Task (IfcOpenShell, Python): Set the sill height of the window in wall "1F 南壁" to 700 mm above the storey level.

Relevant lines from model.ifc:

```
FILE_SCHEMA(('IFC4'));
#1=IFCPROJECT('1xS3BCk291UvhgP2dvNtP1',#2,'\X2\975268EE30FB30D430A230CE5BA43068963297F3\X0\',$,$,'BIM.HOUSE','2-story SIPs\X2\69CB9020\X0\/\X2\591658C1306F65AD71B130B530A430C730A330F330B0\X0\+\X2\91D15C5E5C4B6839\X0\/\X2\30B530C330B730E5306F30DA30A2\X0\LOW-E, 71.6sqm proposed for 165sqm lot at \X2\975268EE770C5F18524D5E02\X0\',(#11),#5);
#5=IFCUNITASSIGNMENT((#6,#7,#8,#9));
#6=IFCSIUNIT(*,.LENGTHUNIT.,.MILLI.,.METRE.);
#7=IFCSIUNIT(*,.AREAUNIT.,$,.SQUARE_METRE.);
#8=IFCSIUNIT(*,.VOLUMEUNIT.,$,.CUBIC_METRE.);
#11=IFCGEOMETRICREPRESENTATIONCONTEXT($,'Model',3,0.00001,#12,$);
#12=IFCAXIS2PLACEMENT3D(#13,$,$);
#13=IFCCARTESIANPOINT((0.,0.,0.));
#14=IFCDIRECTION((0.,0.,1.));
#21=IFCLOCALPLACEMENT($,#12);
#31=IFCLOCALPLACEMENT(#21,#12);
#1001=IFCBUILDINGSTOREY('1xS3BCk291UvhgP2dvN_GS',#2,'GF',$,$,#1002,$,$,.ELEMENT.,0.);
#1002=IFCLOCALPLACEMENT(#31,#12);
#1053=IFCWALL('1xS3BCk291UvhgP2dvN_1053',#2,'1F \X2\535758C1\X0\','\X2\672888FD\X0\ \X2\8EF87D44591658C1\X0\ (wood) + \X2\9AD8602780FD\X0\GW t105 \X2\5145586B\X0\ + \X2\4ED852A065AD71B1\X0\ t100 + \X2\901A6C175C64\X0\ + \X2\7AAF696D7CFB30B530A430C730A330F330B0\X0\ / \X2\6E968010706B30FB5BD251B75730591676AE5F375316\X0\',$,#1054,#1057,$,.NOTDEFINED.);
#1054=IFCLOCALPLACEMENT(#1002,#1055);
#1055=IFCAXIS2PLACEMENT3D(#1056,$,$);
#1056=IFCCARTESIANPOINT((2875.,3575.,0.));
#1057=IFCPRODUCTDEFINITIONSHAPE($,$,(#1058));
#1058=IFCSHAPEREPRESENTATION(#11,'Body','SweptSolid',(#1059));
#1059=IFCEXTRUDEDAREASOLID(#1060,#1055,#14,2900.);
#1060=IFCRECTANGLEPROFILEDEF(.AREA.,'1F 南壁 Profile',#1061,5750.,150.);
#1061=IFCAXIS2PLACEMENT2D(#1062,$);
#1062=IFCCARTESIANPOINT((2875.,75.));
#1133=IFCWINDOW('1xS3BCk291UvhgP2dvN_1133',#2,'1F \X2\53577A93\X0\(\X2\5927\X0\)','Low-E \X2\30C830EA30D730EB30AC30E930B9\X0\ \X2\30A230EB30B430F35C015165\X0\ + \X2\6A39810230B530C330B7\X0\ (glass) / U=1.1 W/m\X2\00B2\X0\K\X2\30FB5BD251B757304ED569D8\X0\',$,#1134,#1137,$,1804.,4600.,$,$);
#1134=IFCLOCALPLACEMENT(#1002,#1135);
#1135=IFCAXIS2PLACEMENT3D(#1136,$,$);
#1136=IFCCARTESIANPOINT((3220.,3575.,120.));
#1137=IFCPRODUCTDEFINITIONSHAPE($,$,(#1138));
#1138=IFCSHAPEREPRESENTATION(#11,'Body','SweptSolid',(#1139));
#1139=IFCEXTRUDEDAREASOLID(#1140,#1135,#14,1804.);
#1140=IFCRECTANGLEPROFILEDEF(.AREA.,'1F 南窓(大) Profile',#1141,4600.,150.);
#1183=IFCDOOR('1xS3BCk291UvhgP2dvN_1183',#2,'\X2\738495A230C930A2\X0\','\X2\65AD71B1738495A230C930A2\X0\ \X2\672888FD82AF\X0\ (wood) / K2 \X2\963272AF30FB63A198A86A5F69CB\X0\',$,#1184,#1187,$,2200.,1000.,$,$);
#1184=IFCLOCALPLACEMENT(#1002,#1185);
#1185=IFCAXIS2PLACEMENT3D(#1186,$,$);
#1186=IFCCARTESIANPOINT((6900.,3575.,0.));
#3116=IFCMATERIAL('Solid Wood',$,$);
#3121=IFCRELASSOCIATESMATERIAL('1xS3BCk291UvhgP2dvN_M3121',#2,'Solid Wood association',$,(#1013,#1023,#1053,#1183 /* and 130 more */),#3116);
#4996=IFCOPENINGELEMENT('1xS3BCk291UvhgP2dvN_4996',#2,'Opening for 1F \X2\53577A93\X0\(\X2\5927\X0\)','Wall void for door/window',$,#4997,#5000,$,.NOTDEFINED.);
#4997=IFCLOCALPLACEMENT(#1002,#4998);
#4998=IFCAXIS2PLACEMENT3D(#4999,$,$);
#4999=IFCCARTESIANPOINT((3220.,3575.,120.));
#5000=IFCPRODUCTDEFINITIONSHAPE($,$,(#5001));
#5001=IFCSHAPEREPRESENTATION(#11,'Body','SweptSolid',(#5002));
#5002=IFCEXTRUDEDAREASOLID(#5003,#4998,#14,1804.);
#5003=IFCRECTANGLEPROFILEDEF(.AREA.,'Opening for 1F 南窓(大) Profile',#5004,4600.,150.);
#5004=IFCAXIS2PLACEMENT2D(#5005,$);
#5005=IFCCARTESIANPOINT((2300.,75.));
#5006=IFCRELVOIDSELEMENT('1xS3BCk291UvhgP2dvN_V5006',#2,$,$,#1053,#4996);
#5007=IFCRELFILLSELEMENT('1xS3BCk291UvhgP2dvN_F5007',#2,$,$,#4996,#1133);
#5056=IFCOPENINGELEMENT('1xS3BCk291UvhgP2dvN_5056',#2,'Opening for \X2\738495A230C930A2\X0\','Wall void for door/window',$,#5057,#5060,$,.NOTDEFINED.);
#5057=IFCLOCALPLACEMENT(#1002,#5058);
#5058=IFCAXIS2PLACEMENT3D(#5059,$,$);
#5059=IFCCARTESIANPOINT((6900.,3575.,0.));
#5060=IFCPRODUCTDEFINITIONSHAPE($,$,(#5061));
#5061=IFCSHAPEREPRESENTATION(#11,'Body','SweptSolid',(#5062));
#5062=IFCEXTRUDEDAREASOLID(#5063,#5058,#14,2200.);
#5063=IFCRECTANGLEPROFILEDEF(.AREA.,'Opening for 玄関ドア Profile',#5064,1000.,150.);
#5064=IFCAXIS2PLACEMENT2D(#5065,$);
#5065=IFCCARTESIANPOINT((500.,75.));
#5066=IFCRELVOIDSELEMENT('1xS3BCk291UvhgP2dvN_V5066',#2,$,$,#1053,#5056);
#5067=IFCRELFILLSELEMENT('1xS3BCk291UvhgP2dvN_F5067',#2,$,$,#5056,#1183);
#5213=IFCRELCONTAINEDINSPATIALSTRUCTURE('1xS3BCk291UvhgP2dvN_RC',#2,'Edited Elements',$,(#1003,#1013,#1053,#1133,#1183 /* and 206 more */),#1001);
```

```python
import numpy as np
import ifcopenshell
import ifcopenshell.api.geometry
import ifcopenshell.geom
import ifcopenshell.util.element
import ifcopenshell.util.placement
import ifcopenshell.util.shape
import ifcopenshell.util.unit

model = ifcopenshell.open("model.ifc")
unit_scale = ifcopenshell.util.unit.calculate_unit_scale(model)

window = model.by_guid("1xS3BCk291UvhgP2dvN_1133")
opening = window.FillsVoids[0].RelatingOpeningElement
storey = ifcopenshell.util.element.get_container(window, ifc_class="IfcBuildingStorey")
level = ifcopenshell.util.placement.get_local_placement(storey.ObjectPlacement)[2, 3]

# The opening's origin need not be at the sill, so measure its lowest point.
shape = ifcopenshell.geom.create_shape(ifcopenshell.geom.settings(), opening)
bottom = ifcopenshell.util.shape.get_shape_bottom_elevation(shape, shape.geometry) / unit_scale
dz = level + 0.7 / unit_scale - bottom

shift = np.array([0.0, 0.0, dz])
# The window is not placed relative to its opening, so move both.
for product in (opening, window):
    matrix = ifcopenshell.util.placement.get_local_placement(product.ObjectPlacement)
    matrix[:3, 3] += shift
    ifcopenshell.api.geometry.edit_object_placement(model, product=product, matrix=matrix, is_si=False)

print(f"moved by {dz * unit_scale:+.3f} m")

model.write("model_v2.ifc")
```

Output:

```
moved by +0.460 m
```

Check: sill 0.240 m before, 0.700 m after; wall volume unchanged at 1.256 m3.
